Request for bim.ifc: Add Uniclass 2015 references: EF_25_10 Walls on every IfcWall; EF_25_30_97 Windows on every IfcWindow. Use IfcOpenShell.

First a look at what the model holds.

```python
import ifcopenshell

model = ifcopenshell.open("bim.ifc")
print(model.schema)
print("classifications:", [c.Name for c in model.by_type("IfcClassification")])
for ifc_class in ("IfcDoor", "IfcRoof", "IfcStair", "IfcWall", "IfcWindow"):
    print(ifc_class, len(model.by_type(ifc_class)))
```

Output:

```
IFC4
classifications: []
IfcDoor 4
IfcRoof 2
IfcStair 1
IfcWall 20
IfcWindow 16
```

```python
import ifcopenshell
import ifcopenshell.api.classification

model = ifcopenshell.open("bim.ifc")

system = ifcopenshell.api.classification.add_classification(model, classification="Uniclass 2015")

codes = {
    "IfcWall": ("EF_25_10", "Walls"),
    "IfcWindow": ("EF_25_30_97", "Windows"),
}
for ifc_class, (code, name) in codes.items():
    products = model.by_type(ifc_class)
    ifcopenshell.api.classification.add_reference(
        model, products=products, classification=system, identification=code, name=name
    )
    print(code, len(products))

model.write("bim_rev.ifc")
```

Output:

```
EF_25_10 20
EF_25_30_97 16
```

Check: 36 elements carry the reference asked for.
